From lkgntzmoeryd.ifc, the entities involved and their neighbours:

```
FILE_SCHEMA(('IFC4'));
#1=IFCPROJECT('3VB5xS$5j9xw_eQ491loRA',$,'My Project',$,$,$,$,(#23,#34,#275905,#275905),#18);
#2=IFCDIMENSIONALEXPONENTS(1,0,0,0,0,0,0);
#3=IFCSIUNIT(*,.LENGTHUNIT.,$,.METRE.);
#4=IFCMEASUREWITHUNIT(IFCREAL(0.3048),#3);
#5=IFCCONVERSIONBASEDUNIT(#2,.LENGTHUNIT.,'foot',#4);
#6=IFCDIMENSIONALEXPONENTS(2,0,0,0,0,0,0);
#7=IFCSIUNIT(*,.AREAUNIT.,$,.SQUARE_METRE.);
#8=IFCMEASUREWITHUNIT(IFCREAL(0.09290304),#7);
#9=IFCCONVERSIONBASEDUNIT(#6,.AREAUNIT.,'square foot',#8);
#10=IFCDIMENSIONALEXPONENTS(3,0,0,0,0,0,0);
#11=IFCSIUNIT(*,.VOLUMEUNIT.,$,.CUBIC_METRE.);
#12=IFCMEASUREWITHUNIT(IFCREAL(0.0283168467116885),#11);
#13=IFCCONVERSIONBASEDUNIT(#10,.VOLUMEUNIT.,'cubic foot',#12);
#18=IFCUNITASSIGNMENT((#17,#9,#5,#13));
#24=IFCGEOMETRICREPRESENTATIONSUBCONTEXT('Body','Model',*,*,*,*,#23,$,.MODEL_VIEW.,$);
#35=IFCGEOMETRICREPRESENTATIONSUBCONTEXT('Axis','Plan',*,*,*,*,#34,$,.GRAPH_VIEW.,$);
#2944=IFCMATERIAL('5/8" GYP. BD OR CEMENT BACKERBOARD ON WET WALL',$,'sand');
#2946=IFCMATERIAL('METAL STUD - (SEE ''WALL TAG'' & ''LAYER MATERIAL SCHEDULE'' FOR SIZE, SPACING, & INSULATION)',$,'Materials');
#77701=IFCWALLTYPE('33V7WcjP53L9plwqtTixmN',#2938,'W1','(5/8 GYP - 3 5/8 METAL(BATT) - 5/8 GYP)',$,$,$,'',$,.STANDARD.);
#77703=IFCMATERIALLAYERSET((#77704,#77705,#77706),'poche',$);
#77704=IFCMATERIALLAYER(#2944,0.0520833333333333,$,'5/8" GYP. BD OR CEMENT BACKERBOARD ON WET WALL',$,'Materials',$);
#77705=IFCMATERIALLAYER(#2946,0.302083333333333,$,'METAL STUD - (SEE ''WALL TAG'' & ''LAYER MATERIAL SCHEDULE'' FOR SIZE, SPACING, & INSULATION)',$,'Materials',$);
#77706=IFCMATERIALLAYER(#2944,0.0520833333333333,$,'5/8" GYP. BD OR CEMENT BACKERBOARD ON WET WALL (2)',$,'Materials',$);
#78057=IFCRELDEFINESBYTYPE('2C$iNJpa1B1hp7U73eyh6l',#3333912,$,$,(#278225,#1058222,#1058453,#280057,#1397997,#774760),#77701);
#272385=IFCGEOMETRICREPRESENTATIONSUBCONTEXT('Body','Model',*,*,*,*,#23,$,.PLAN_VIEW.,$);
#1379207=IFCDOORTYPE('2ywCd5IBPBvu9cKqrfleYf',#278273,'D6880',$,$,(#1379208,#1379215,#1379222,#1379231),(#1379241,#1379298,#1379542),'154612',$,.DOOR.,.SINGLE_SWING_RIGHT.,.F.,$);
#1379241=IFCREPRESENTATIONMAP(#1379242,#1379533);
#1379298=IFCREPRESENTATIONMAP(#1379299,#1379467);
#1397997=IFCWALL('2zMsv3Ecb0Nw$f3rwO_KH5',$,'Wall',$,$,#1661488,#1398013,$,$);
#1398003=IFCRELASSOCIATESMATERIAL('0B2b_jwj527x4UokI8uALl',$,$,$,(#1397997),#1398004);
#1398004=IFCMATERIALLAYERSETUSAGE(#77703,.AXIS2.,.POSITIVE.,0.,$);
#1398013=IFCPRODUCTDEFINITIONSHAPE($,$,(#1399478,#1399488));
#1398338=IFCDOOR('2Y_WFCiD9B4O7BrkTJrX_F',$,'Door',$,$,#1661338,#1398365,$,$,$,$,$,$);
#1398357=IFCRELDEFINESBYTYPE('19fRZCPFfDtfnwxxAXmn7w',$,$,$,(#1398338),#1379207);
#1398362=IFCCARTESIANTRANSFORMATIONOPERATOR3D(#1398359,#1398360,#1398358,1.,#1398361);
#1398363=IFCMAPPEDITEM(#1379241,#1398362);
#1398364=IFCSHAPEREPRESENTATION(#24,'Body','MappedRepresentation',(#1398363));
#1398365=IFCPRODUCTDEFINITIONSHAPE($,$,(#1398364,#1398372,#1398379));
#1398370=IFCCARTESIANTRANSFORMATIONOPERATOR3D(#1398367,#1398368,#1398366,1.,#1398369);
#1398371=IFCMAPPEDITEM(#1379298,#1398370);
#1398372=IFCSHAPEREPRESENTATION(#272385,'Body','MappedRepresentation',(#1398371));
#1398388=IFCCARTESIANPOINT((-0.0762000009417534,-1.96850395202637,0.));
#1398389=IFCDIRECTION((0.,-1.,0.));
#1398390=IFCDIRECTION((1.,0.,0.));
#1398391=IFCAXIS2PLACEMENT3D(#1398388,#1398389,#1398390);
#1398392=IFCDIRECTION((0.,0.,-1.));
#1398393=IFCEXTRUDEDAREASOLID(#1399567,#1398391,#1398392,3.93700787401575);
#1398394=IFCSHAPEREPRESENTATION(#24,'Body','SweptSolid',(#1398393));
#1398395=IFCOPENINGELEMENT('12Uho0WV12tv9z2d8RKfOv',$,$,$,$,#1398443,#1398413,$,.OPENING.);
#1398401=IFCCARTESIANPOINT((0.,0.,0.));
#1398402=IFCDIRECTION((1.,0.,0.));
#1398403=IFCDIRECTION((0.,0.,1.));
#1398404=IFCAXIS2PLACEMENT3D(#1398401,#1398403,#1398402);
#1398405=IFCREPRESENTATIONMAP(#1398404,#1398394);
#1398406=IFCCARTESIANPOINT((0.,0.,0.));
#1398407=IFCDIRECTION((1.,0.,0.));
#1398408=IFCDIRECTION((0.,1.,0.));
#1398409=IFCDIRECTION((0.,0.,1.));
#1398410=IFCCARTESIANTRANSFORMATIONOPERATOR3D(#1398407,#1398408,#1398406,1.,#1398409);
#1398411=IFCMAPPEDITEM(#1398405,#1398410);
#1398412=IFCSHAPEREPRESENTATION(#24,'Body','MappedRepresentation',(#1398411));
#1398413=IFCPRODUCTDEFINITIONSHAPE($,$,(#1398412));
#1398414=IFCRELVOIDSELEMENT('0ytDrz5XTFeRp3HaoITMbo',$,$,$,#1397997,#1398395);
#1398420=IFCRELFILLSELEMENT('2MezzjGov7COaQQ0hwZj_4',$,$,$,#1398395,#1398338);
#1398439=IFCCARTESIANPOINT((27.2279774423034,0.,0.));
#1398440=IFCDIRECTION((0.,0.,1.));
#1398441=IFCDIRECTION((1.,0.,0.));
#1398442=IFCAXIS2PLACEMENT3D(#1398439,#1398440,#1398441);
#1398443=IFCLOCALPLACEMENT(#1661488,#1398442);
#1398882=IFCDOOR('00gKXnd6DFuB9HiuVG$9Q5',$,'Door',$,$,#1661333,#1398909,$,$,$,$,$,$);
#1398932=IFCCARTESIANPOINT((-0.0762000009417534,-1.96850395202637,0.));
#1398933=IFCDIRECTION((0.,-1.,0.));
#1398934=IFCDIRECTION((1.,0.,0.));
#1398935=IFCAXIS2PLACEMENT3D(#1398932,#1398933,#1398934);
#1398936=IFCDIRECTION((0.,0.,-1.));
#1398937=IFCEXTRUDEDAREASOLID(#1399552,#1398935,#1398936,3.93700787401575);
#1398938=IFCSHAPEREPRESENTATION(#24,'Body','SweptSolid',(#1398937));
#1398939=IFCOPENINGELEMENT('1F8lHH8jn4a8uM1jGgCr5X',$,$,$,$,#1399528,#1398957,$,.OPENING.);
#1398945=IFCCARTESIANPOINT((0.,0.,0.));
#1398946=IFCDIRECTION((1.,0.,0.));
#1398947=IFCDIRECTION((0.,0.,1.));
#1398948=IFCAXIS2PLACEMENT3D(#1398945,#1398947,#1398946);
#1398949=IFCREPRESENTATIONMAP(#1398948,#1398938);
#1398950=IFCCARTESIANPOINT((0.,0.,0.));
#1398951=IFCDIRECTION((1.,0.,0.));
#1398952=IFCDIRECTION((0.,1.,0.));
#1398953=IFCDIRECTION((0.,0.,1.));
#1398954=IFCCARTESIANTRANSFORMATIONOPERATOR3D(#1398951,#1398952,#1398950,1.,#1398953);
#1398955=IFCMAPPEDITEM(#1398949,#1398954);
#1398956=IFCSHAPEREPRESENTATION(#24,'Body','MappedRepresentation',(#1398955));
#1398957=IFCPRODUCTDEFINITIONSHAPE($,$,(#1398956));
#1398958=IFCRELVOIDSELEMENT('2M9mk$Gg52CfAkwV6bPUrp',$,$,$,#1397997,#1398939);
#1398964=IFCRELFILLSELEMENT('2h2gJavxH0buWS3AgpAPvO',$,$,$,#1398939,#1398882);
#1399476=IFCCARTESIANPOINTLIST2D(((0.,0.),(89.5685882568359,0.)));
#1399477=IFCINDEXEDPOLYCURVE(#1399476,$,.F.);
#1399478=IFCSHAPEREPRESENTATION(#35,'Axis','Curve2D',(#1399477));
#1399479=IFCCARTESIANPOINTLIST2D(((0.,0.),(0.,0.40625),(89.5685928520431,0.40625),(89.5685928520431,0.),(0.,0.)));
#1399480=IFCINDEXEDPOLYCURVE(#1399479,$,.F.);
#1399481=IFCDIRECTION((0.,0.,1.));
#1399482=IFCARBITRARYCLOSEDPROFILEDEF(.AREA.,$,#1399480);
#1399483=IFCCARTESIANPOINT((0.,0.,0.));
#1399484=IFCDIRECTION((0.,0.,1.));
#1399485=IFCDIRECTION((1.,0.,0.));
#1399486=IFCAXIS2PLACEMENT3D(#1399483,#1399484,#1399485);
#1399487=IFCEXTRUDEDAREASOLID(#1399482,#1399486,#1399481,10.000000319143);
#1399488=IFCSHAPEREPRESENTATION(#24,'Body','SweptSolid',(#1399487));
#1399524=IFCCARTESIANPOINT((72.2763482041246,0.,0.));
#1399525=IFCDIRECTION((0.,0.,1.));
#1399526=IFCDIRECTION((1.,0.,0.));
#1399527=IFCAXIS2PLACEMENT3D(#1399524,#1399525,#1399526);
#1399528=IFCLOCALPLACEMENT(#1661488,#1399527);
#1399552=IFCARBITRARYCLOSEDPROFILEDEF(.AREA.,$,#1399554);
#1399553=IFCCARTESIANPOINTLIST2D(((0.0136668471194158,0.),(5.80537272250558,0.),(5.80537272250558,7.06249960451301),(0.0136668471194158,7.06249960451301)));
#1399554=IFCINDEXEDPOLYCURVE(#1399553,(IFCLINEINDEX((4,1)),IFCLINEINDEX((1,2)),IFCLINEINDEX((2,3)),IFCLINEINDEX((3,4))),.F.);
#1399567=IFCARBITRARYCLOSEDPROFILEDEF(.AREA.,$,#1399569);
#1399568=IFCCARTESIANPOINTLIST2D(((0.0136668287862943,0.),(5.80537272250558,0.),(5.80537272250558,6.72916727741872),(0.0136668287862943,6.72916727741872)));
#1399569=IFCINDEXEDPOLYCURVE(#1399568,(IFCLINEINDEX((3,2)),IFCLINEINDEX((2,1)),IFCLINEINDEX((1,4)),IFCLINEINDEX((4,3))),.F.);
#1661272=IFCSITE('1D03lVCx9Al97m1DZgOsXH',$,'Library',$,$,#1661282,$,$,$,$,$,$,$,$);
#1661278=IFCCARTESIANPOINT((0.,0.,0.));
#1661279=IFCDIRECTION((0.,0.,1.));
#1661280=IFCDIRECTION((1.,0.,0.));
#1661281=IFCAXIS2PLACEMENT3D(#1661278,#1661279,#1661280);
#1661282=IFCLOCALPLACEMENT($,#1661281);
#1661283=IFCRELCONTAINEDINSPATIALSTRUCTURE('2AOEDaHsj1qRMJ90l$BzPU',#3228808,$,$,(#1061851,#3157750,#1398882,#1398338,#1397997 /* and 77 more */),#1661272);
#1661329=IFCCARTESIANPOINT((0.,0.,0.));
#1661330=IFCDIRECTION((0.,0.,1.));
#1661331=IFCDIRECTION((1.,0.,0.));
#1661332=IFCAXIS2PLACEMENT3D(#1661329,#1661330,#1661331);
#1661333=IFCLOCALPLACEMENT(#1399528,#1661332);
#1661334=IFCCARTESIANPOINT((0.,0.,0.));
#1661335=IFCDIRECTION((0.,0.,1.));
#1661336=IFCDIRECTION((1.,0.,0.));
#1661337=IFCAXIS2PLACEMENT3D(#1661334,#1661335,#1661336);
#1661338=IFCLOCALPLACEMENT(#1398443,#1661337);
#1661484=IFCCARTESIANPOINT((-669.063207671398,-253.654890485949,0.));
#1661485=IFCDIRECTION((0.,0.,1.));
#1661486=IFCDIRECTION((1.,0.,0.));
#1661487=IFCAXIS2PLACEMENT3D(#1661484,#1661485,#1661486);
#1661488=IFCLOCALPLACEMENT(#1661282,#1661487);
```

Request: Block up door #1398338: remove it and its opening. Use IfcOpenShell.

```python
import ifcopenshell
import ifcopenshell.api.feature
import ifcopenshell.api.root
import ifcopenshell.geom
import ifcopenshell.util.shape

model = ifcopenshell.open("lkgntzmoeryd.ifc")
settings = ifcopenshell.geom.settings()


def volume(element):
    """Net volume in cubic metres, openings subtracted."""
    shape = ifcopenshell.geom.create_shape(settings, element)
    return ifcopenshell.util.shape.get_volume(shape.geometry)


door = model.by_guid("2Y_WFCiD9B4O7BrkTJrX_F")
opening = door.FillsVoids[0].RelatingOpeningElement
wall = opening.VoidsElements[0].RelatingBuildingElement
before = volume(wall)

ifcopenshell.api.root.remove_product(model, product=door)
ifcopenshell.api.feature.remove_feature(model, feature=opening)

after = volume(wall)

print(f"wall volume {before:.3f} -> {after:.3f} m3")

model.write("lkgntzmoeryd_v2.ifc")
```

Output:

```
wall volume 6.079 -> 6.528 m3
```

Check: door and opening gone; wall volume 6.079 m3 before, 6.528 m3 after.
